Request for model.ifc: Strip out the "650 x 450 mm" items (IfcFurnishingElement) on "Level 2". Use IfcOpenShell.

First a look at what the model holds.

```python
import ifcopenshell
import ifcopenshell.util.element

model = ifcopenshell.open("model.ifc")
print(model.schema)
storey = next(s for s in model.by_type("IfcBuildingStorey") if s.Name == "Level 2")
furniture = [e for e in ifcopenshell.util.element.get_decomposition(storey) if e.is_a("IfcFurnishingElement")]
seen = {}
for e in furniture:
    element_type = ifcopenshell.util.element.get_type(e)
    name = element_type.Name if element_type not in (None, e) else None
    seen[name] = seen.get(name, 0) + 1
for name, count in sorted(seen.items(), key=str):
    print(count, "x", name)
```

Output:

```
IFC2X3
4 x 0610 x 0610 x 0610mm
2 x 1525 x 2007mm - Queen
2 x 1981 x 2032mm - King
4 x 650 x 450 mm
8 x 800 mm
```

```python
import ifcopenshell
import ifcopenshell.api.root
import ifcopenshell.util.element

model = ifcopenshell.open("model.ifc")

storey = next(s for s in model.by_type("IfcBuildingStorey") if s.Name == "Level 2")
furniture = [e for e in ifcopenshell.util.element.get_decomposition(storey) if e.is_a("IfcFurnishingElement")]
targets = [e for e in furniture if (t := ifcopenshell.util.element.get_type(e)) not in (None, e) and t.Name == "650 x 450 mm"]

for e in targets:
    ifcopenshell.api.root.remove_product(model, product=e)
print(len(targets), "removed")

model.write("model_rev.ifc")
```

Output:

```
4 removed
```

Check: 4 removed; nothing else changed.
